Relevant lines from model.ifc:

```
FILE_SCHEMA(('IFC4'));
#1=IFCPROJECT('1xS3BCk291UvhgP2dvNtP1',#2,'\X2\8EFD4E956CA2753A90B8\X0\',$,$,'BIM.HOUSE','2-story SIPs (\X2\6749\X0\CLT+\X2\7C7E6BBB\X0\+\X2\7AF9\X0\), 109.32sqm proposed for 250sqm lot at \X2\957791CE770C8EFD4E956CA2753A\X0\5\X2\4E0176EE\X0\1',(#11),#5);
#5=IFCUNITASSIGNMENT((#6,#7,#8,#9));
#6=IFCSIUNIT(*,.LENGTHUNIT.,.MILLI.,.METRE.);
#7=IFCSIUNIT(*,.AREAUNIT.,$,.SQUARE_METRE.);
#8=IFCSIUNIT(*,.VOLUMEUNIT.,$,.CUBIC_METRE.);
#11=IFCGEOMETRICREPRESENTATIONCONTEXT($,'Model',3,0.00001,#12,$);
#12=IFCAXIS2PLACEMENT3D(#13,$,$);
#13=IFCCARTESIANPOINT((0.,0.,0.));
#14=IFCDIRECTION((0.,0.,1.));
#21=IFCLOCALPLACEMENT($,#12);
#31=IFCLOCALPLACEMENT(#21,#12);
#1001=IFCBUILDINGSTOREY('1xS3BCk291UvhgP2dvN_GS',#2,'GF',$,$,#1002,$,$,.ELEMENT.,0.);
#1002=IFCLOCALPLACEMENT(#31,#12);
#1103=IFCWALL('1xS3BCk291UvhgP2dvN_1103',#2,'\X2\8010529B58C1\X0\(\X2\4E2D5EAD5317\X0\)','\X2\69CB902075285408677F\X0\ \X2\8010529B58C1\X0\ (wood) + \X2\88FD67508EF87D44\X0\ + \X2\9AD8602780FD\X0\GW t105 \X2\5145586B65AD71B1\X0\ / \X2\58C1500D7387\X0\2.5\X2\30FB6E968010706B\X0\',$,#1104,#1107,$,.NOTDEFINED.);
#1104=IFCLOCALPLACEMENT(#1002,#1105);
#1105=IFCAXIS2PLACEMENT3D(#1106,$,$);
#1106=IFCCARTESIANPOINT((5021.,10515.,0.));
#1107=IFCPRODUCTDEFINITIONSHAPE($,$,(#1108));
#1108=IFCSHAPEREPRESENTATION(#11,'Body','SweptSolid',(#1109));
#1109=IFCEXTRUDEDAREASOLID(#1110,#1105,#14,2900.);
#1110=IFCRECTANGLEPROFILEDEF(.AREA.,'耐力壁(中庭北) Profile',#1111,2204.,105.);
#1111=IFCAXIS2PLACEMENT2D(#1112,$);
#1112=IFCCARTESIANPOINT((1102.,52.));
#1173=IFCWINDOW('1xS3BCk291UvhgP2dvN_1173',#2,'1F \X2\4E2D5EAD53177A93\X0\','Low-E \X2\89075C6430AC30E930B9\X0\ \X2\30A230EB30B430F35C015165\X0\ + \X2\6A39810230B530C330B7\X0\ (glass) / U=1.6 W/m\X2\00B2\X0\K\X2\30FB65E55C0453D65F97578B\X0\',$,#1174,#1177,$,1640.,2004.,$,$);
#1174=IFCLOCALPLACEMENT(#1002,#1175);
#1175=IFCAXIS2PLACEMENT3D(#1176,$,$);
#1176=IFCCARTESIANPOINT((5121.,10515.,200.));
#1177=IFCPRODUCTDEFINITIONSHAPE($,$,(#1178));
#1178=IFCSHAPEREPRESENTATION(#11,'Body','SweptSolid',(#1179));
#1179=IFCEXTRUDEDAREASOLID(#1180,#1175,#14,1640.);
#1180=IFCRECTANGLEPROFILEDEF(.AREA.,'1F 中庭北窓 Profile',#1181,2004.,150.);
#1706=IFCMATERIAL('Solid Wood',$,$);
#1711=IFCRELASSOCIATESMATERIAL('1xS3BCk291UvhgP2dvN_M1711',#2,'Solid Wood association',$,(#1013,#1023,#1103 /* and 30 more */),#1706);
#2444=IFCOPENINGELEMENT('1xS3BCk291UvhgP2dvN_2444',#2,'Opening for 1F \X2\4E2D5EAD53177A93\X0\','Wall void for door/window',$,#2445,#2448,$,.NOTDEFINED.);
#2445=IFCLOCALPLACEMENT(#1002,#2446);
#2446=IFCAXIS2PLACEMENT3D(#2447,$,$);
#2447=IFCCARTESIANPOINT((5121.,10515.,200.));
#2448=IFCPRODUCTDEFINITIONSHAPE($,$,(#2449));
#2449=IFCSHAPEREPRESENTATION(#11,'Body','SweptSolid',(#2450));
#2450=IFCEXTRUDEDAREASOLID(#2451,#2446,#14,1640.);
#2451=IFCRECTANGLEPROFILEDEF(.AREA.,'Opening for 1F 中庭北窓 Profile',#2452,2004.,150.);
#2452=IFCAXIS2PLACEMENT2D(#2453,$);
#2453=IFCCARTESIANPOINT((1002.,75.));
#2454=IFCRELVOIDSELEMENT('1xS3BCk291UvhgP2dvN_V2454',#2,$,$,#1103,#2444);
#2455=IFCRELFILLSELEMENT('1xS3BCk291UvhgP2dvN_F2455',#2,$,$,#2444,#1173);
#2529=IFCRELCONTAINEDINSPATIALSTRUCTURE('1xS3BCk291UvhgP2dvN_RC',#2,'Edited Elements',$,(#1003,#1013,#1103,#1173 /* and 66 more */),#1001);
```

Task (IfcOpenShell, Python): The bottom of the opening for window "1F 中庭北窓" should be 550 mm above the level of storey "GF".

```python
import numpy as np
import ifcopenshell
import ifcopenshell.api.geometry
import ifcopenshell.geom
import ifcopenshell.util.element
import ifcopenshell.util.placement
import ifcopenshell.util.shape
import ifcopenshell.util.unit

model = ifcopenshell.open("model.ifc")
unit_scale = ifcopenshell.util.unit.calculate_unit_scale(model)

window = model.by_id(1173)
opening = window.FillsVoids[0].RelatingOpeningElement
storey = ifcopenshell.util.element.get_container(window, ifc_class="IfcBuildingStorey")
level = ifcopenshell.util.placement.get_local_placement(storey.ObjectPlacement)[2, 3]

# The opening's origin need not be at the sill, so measure its lowest point.
shape = ifcopenshell.geom.create_shape(ifcopenshell.geom.settings(), opening)
bottom = ifcopenshell.util.shape.get_shape_bottom_elevation(shape, shape.geometry) / unit_scale
dz = level + 0.55 / unit_scale - bottom

shift = np.array([0.0, 0.0, dz])
# The window is not placed relative to its opening, so move both.
for product in (opening, window):
    matrix = ifcopenshell.util.placement.get_local_placement(product.ObjectPlacement)
    matrix[:3, 3] += shift
    ifcopenshell.api.geometry.edit_object_placement(model, product=product, matrix=matrix, is_si=False)

print(f"moved by {dz * unit_scale:+.3f} m")

model.write("model_v2.ifc")
```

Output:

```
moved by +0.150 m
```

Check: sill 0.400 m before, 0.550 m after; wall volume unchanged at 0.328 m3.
